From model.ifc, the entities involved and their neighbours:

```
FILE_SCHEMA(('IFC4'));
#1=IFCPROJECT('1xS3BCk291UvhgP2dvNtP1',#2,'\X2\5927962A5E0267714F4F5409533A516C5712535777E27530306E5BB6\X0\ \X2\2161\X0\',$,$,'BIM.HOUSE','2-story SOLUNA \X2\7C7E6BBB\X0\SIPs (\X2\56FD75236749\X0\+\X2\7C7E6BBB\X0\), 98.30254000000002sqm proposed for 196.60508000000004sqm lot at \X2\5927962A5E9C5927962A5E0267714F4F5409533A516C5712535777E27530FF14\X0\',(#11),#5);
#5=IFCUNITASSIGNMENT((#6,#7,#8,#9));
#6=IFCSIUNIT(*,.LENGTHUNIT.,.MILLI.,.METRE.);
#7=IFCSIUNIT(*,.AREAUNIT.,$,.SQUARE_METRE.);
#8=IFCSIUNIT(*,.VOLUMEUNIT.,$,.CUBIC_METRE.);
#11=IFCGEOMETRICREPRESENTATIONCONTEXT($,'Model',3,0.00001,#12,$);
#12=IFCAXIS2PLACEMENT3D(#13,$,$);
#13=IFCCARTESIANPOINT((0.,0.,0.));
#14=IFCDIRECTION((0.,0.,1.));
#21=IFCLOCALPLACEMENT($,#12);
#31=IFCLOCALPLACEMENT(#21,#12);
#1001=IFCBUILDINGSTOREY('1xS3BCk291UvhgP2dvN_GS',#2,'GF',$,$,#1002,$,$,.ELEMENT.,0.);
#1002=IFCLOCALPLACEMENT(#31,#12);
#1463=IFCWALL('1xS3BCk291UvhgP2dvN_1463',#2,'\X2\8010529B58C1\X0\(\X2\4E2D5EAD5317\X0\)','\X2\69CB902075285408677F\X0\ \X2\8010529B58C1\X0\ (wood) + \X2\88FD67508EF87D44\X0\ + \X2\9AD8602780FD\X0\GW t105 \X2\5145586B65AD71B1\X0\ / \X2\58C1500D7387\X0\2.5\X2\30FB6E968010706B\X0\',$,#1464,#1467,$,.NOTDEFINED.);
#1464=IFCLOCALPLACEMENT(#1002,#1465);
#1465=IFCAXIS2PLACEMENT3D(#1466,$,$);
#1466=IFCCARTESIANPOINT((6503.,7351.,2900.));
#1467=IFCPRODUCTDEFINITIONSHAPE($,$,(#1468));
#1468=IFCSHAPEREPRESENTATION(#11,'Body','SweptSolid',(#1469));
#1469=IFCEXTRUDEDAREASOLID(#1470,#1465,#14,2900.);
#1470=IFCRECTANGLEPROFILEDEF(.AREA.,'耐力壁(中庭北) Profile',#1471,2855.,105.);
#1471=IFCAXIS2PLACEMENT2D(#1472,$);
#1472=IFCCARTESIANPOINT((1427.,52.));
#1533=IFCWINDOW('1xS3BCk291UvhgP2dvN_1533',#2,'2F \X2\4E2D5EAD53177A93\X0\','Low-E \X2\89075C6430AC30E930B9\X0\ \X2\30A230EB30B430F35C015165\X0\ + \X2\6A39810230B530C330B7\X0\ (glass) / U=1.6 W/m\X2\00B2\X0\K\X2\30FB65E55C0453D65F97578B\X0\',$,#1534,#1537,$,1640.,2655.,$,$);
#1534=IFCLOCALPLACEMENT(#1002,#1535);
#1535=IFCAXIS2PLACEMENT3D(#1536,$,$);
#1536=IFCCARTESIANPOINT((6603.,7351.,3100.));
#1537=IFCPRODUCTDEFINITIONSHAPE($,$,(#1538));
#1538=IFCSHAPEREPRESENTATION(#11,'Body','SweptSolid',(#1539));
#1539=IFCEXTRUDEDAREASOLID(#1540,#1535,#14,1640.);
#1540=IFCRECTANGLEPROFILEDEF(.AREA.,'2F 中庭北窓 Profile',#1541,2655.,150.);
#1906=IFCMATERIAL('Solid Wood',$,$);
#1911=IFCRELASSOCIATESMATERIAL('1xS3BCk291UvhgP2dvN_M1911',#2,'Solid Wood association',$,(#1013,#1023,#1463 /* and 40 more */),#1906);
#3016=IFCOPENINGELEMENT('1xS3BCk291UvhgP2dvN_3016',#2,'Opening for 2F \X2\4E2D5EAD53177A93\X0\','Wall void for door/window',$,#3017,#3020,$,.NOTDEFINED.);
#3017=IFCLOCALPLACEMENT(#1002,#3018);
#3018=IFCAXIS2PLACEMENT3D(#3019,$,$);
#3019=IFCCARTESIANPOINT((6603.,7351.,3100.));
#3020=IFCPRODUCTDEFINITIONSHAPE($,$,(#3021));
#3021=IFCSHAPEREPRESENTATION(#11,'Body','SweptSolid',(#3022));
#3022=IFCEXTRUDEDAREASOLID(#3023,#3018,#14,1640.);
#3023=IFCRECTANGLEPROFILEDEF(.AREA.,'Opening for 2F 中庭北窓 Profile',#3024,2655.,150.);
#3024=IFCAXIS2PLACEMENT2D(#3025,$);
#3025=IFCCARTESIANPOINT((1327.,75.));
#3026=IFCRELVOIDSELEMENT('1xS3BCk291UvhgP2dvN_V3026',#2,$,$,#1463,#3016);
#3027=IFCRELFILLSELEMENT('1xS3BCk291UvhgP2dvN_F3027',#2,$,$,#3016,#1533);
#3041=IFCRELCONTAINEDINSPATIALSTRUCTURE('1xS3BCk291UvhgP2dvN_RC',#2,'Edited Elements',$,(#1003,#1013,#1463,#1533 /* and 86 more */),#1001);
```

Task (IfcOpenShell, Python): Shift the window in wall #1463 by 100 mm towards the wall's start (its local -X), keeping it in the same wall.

```python
import ifcopenshell
import ifcopenshell.api.geometry
import ifcopenshell.util.placement

model = ifcopenshell.open("model.ifc")

window = model.by_guid("1xS3BCk291UvhgP2dvN_1533")
opening = window.FillsVoids[0].RelatingOpeningElement
wall = opening.VoidsElements[0].RelatingBuildingElement

wall_matrix = ifcopenshell.util.placement.get_local_placement(wall.ObjectPlacement)
shift = wall_matrix[:3, 0] * -100.0
before = ifcopenshell.util.placement.get_local_placement(window.ObjectPlacement)[:3, 3].copy()

# The window is not placed relative to its opening, so move both.
for product in (opening, window):
    matrix = ifcopenshell.util.placement.get_local_placement(product.ObjectPlacement)
    matrix[:3, 3] += shift
    ifcopenshell.api.geometry.edit_object_placement(model, product=product, matrix=matrix, is_si=False)

after = ifcopenshell.util.placement.get_local_placement(window.ObjectPlacement)[:3, 3]
print("window moved by", (after - before).round(3) + 0.0)

model.write("model_v2.ifc")
```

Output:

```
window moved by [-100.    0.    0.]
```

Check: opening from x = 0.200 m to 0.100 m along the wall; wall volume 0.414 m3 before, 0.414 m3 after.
